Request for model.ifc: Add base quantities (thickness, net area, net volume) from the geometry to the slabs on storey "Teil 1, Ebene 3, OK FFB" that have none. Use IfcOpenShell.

First a look at what the model holds.

```python
import ifcopenshell
import ifcopenshell.util.element
import ifcopenshell.util.unit

model = ifcopenshell.open("model.ifc")
print(model.schema)
for unit_type in ("LENGTHUNIT", "AREAUNIT", "VOLUMEUNIT"):
    print(unit_type, ifcopenshell.util.unit.calculate_unit_scale(model, unit_type))
storey = next(s for s in model.by_type("IfcBuildingStorey") if s.Name == "Teil 1, Ebene 3, OK FFB")
slabs = [e for e in ifcopenshell.util.element.get_decomposition(storey) if e.is_a("IfcSlab")]
for e in sorted(slabs, key=lambda e: e.id()):
    print(e.id(), e.is_a(), e.Name, list(ifcopenshell.util.element.get_psets(e, qtos_only=True)), sep=" | ")
```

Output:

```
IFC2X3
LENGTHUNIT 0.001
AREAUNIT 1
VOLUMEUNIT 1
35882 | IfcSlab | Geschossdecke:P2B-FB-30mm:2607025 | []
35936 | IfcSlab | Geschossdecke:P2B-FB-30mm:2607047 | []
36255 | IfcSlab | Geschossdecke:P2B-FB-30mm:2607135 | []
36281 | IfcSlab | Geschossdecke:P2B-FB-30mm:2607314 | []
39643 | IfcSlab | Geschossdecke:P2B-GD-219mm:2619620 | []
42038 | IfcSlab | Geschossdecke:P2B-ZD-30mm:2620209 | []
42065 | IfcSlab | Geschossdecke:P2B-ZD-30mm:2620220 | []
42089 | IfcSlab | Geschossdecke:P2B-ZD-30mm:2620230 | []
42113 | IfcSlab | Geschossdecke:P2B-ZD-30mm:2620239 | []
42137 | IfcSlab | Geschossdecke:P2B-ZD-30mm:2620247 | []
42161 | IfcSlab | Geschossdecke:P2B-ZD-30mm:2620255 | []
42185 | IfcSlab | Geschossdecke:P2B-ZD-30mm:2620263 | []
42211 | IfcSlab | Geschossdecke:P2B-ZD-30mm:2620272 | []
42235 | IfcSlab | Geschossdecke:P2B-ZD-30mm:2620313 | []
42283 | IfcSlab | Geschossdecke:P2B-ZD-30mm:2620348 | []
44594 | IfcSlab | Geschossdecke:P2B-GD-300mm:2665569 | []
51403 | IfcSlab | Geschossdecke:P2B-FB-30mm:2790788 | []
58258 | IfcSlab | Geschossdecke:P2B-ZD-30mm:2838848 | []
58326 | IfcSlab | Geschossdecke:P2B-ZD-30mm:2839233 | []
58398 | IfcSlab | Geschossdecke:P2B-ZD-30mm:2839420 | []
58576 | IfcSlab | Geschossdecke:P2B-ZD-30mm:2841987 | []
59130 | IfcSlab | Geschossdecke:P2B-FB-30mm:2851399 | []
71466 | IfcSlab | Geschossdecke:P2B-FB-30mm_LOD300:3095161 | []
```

```python
import ifcopenshell
import ifcopenshell.api.pset
import ifcopenshell.geom
import ifcopenshell.util.element
import ifcopenshell.util.shape
import ifcopenshell.util.unit

model = ifcopenshell.open("model.ifc")
unit_scale = ifcopenshell.util.unit.calculate_unit_scale(model)
area_scale = ifcopenshell.util.unit.calculate_unit_scale(model, "AREAUNIT")
volume_scale = ifcopenshell.util.unit.calculate_unit_scale(model, "VOLUMEUNIT")
settings = ifcopenshell.geom.settings()

storey = next(s for s in model.by_type("IfcBuildingStorey") if s.Name == "Teil 1, Ebene 3, OK FFB")
slabs = [e for e in ifcopenshell.util.element.get_decomposition(storey) if e.is_a("IfcSlab")]

for e in sorted(slabs, key=lambda e: e.id()):
    if ifcopenshell.util.element.get_psets(e, qtos_only=True, should_inherit=False):
        continue
    # Geometry comes back in metres, in the element's own axes.
    shape = ifcopenshell.geom.create_shape(settings, e)
    values = {
        "Width": ifcopenshell.util.shape.get_z(shape.geometry) / unit_scale,
        "NetArea": ifcopenshell.util.shape.get_footprint_area(shape.geometry) / area_scale,
        "NetVolume": ifcopenshell.util.shape.get_volume(shape.geometry) / volume_scale,
    }
    qto = ifcopenshell.api.pset.add_qto(model, product=e, name="BaseQuantities")
    ifcopenshell.api.pset.edit_qto(model, qto=qto, properties=values)
    print(e.id(), {k: round(v, 3) for k, v in values.items()})

model.write("model_edited.ifc")
```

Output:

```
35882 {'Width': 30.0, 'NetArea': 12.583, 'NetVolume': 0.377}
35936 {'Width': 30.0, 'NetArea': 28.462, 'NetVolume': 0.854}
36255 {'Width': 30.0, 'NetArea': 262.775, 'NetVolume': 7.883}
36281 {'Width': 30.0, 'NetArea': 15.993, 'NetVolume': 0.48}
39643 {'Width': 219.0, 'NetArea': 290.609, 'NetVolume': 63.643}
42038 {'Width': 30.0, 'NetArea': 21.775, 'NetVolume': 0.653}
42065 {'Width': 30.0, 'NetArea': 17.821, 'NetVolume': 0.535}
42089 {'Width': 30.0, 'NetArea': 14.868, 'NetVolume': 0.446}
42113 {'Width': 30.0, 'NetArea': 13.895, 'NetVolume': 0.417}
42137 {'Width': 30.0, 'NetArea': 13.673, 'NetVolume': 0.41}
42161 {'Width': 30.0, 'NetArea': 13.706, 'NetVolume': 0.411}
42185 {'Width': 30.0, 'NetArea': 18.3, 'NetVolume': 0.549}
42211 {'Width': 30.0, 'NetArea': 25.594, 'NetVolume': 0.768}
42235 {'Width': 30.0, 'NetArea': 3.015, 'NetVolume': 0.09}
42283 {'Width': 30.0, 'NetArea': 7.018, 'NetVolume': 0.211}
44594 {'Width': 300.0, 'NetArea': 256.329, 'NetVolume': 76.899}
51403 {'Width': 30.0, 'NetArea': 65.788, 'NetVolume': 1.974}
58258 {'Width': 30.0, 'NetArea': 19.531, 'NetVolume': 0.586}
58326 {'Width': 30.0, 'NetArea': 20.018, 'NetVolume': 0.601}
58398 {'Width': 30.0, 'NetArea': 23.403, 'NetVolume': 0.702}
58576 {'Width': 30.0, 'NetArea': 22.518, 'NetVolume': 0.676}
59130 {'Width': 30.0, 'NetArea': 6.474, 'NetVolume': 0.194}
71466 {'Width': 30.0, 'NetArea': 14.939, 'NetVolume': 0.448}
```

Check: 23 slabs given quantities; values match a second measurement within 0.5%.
